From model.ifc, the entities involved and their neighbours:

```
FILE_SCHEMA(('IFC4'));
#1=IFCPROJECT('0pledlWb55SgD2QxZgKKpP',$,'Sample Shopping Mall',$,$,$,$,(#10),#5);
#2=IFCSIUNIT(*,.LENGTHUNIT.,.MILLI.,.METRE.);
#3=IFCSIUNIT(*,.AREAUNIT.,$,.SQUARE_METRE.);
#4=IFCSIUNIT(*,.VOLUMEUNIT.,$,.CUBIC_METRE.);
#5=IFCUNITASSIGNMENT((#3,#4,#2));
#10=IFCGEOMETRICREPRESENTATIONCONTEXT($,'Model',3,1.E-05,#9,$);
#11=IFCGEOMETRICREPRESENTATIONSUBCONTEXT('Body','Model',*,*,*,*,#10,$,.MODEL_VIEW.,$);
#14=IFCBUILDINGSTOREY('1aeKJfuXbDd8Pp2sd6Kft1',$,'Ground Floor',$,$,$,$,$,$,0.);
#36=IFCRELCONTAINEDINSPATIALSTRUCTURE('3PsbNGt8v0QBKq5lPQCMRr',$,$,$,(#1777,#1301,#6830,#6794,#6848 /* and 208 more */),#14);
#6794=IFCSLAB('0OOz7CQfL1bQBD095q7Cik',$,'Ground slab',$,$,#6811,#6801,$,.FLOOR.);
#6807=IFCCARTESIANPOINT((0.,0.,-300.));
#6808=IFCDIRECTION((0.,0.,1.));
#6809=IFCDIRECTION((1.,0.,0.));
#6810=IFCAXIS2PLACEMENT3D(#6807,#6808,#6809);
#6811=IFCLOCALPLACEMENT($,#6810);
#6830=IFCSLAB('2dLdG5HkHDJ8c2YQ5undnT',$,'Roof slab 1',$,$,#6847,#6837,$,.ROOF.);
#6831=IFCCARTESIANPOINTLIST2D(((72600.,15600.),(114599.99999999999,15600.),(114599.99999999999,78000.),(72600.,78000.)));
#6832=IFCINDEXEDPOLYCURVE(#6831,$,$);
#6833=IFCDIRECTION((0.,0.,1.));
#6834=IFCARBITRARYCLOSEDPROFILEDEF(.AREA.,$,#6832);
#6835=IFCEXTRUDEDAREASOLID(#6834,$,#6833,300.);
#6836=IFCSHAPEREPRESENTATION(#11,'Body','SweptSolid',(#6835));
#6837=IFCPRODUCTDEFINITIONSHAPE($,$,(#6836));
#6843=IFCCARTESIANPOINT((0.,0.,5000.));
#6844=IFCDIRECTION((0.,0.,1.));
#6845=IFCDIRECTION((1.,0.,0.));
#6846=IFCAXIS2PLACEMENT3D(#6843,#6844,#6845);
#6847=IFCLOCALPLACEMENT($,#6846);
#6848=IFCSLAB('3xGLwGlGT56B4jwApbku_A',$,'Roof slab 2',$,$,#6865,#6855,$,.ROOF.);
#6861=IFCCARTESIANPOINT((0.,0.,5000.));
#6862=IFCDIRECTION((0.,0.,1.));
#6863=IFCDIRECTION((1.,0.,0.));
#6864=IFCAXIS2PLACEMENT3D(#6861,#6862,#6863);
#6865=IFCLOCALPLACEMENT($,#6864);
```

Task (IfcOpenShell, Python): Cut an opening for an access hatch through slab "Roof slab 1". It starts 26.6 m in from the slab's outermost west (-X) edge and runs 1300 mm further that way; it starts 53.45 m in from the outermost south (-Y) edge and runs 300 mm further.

```python
import numpy as np
import ifcopenshell
import ifcopenshell.api.feature
import ifcopenshell.api.geometry
import ifcopenshell.api.root
import ifcopenshell.geom
import ifcopenshell.util.placement
import ifcopenshell.util.representation
import ifcopenshell.util.shape
import ifcopenshell.util.unit

model = ifcopenshell.open("model.ifc")
unit_scale = ifcopenshell.util.unit.calculate_unit_scale(model)
settings = ifcopenshell.geom.settings()


def volume(element):
    """Net volume in cubic metres, openings subtracted."""
    shape = ifcopenshell.geom.create_shape(settings, element)
    return ifcopenshell.util.shape.get_volume(shape.geometry)


slab = model.by_guid("2dLdG5HkHDJ8c2YQ5undnT")
before = volume(slab)

# Extent in the slab's own axes, in metres. The edges named are its -X and -Y sides.
slab_shape = ifcopenshell.geom.create_shape(settings, slab)
vertices = ifcopenshell.util.shape.get_vertices(slab_shape.geometry)
x_min, y_min, bottom = vertices.min(axis=0)
top = vertices[:, 2].max()

opening = ifcopenshell.api.root.create_entity(model, ifc_class="IfcOpeningElement", name="Access hatch opening", predefined_type="OPENING")
context = ifcopenshell.util.representation.get_context(model, "Model", "Body", "MODEL_VIEW")
width, depth = 1.3, 0.3
outline = [(0.0, 0.0), (width, 0.0), (width, depth), (0.0, depth), (0.0, 0.0)]
# Overshoot both faces by 50 mm so the cut is clean.
shape = ifcopenshell.api.geometry.add_slab_representation(
    model, context=context, depth=top - bottom + 0.1, polyline=outline
)
ifcopenshell.api.geometry.assign_representation(model, product=opening, representation=shape)

matrix = ifcopenshell.util.placement.get_local_placement(slab.ObjectPlacement)
matrix[:, 3] = matrix @ np.append(np.array([x_min + 26.6, y_min + 53.45, bottom - 0.05]) / unit_scale, 1.0)
ifcopenshell.api.geometry.edit_object_placement(model, product=opening, matrix=matrix, is_si=False)
ifcopenshell.api.feature.add_feature(model, feature=opening, element=slab)

after = volume(slab)

print(f"slab volume {before:.3f} -> {after:.3f} m3")

model.write("model-out.ifc")
```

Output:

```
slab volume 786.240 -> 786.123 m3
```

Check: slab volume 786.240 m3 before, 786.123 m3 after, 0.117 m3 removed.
